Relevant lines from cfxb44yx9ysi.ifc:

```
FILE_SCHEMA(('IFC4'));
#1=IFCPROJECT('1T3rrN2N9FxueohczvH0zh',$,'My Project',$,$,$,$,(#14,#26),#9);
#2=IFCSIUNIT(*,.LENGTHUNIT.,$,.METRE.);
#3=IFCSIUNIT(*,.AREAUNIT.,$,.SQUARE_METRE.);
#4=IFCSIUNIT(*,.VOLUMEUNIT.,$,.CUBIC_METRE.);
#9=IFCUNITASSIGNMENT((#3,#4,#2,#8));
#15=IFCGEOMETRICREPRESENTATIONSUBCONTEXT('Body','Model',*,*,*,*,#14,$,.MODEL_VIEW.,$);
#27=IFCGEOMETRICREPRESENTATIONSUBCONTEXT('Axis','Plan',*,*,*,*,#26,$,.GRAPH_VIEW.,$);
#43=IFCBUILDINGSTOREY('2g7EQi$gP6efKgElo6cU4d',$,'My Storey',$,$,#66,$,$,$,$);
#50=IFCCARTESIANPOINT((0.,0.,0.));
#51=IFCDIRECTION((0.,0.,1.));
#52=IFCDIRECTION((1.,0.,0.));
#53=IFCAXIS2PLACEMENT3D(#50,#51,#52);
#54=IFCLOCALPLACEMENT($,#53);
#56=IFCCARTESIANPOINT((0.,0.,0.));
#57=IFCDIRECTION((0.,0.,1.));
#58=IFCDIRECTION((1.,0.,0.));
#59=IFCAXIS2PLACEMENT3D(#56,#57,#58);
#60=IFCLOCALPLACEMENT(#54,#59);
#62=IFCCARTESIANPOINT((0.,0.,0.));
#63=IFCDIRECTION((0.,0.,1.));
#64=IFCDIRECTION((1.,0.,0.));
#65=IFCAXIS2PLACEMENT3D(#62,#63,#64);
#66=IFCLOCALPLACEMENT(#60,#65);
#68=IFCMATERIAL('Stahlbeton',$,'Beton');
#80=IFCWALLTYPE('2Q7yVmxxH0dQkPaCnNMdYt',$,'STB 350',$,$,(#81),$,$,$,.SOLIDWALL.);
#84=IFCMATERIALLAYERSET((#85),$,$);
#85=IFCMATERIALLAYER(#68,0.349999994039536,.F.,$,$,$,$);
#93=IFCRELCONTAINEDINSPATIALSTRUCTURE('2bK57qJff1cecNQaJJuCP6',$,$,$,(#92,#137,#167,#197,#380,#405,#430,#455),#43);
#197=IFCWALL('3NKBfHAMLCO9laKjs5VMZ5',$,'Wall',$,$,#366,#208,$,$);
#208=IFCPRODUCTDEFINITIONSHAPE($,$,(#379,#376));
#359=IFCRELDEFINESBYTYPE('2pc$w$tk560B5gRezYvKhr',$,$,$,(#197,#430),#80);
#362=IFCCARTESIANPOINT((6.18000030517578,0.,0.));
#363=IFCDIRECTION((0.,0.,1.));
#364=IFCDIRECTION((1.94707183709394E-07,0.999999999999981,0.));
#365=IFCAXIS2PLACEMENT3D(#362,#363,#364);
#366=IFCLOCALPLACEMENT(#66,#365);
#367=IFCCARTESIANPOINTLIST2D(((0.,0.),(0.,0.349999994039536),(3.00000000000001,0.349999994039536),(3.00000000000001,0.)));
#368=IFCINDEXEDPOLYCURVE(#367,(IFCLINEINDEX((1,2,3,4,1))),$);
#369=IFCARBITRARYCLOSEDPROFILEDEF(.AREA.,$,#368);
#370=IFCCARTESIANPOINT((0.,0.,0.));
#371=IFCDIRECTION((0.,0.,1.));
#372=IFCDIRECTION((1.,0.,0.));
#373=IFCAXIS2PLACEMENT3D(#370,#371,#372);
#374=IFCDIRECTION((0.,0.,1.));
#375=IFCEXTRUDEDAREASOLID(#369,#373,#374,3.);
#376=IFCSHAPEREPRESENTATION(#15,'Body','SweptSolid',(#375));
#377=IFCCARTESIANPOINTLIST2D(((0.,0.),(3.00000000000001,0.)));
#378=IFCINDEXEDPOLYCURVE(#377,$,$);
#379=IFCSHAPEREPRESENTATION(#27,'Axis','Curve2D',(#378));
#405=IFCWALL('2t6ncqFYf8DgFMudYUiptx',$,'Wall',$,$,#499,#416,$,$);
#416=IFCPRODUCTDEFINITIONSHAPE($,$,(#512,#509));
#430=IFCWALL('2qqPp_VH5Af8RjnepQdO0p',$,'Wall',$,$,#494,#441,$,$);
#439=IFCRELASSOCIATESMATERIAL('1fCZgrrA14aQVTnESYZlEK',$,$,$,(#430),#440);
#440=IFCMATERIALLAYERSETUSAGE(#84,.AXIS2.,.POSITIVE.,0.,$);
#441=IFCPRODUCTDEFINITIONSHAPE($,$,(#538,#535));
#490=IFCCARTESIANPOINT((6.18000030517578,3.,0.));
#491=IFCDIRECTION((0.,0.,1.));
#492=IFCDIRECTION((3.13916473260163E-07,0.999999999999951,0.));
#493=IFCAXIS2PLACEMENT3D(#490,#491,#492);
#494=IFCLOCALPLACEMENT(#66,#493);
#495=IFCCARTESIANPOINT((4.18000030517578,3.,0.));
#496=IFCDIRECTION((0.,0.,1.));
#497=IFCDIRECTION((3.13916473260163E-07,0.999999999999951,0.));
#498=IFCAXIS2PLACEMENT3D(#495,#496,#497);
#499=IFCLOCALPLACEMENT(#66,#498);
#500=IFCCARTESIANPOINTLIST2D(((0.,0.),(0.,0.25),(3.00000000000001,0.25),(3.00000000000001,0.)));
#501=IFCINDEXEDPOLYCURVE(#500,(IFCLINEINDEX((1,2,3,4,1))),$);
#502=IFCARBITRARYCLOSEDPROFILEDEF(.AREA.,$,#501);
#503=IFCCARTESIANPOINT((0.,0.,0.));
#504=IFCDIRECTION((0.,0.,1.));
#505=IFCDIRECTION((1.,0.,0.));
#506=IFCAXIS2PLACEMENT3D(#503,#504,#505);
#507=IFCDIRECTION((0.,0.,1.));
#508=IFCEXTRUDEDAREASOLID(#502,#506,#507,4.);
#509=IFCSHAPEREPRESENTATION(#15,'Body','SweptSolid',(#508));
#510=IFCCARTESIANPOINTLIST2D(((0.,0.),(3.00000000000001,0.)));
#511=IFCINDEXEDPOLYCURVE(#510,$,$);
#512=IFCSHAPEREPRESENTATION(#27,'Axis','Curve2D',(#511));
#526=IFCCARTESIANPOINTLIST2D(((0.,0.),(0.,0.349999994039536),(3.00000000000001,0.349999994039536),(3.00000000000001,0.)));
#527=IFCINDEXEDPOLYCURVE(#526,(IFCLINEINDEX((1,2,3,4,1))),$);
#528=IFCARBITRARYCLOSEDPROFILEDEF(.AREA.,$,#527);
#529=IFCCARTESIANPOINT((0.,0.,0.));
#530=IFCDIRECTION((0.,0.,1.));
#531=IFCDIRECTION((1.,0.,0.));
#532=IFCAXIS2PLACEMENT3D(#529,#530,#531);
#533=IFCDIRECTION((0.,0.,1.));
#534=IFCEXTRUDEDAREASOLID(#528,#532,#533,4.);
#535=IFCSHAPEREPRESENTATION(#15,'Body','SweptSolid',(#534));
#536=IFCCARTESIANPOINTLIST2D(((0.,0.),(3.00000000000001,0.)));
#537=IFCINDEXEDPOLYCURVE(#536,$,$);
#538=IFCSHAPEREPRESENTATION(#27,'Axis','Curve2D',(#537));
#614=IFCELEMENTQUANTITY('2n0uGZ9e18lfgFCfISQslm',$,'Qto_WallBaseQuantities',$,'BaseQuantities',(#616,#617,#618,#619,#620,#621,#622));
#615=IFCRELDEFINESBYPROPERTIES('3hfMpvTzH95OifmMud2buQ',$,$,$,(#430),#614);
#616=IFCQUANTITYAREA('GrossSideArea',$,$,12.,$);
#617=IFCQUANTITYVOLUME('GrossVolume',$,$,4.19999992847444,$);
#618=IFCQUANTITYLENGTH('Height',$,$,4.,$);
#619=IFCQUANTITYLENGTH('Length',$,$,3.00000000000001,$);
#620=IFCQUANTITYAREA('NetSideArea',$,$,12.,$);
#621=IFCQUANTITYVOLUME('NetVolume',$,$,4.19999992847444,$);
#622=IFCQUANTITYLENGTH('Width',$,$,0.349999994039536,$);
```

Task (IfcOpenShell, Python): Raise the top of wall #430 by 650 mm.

```python
import ifcopenshell
import ifcopenshell.api.pset
import ifcopenshell.geom
import ifcopenshell.util.element
import ifcopenshell.util.representation
import ifcopenshell.util.shape
import ifcopenshell.util.unit

model = ifcopenshell.open("cfxb44yx9ysi.ifc")
unit_scale = ifcopenshell.util.unit.calculate_unit_scale(model)
area_scale = ifcopenshell.util.unit.calculate_unit_scale(model, "AREAUNIT")
volume_scale = ifcopenshell.util.unit.calculate_unit_scale(model, "VOLUMEUNIT")
settings = ifcopenshell.geom.settings()


def volume(element):
    """Net volume in cubic metres, openings subtracted."""
    shape = ifcopenshell.geom.create_shape(settings, element)
    return ifcopenshell.util.shape.get_volume(shape.geometry)


wall = model.by_guid("2qqPp_VH5Af8RjnepQdO0p")
before = volume(wall)

body = ifcopenshell.util.representation.get_representation(wall, "Model", "Body")
solid = body.Items[0]
old_height = solid.Depth
solid.Depth += 0.65
after = volume(wall)
thickness = 0.35  # wall thickness in metres

# Update the stored height, areas and volumes.
qto = model.by_id(ifcopenshell.util.element.get_pset(wall, "Qto_WallBaseQuantities", should_inherit=False)["id"])
ifcopenshell.api.pset.edit_qto(model, qto=qto, properties={
    "GrossSideArea": ifcopenshell.util.element.get_pset(wall, "Qto_WallBaseQuantities", "GrossSideArea") * solid.Depth / old_height,
    "GrossVolume": ifcopenshell.util.element.get_pset(wall, "Qto_WallBaseQuantities", "GrossVolume") * solid.Depth / old_height,
    "Height": solid.Depth,
    "NetSideArea": after / thickness / area_scale,
    "NetVolume": after / volume_scale,
})

print(f"height {old_height:g} -> {solid.Depth:g}, volume {before:.3f} -> {after:.3f} m3")

model.write("cfxb44yx9ysi_updated.ifc")
```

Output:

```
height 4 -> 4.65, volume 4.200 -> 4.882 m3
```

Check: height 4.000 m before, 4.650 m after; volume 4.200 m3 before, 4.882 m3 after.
